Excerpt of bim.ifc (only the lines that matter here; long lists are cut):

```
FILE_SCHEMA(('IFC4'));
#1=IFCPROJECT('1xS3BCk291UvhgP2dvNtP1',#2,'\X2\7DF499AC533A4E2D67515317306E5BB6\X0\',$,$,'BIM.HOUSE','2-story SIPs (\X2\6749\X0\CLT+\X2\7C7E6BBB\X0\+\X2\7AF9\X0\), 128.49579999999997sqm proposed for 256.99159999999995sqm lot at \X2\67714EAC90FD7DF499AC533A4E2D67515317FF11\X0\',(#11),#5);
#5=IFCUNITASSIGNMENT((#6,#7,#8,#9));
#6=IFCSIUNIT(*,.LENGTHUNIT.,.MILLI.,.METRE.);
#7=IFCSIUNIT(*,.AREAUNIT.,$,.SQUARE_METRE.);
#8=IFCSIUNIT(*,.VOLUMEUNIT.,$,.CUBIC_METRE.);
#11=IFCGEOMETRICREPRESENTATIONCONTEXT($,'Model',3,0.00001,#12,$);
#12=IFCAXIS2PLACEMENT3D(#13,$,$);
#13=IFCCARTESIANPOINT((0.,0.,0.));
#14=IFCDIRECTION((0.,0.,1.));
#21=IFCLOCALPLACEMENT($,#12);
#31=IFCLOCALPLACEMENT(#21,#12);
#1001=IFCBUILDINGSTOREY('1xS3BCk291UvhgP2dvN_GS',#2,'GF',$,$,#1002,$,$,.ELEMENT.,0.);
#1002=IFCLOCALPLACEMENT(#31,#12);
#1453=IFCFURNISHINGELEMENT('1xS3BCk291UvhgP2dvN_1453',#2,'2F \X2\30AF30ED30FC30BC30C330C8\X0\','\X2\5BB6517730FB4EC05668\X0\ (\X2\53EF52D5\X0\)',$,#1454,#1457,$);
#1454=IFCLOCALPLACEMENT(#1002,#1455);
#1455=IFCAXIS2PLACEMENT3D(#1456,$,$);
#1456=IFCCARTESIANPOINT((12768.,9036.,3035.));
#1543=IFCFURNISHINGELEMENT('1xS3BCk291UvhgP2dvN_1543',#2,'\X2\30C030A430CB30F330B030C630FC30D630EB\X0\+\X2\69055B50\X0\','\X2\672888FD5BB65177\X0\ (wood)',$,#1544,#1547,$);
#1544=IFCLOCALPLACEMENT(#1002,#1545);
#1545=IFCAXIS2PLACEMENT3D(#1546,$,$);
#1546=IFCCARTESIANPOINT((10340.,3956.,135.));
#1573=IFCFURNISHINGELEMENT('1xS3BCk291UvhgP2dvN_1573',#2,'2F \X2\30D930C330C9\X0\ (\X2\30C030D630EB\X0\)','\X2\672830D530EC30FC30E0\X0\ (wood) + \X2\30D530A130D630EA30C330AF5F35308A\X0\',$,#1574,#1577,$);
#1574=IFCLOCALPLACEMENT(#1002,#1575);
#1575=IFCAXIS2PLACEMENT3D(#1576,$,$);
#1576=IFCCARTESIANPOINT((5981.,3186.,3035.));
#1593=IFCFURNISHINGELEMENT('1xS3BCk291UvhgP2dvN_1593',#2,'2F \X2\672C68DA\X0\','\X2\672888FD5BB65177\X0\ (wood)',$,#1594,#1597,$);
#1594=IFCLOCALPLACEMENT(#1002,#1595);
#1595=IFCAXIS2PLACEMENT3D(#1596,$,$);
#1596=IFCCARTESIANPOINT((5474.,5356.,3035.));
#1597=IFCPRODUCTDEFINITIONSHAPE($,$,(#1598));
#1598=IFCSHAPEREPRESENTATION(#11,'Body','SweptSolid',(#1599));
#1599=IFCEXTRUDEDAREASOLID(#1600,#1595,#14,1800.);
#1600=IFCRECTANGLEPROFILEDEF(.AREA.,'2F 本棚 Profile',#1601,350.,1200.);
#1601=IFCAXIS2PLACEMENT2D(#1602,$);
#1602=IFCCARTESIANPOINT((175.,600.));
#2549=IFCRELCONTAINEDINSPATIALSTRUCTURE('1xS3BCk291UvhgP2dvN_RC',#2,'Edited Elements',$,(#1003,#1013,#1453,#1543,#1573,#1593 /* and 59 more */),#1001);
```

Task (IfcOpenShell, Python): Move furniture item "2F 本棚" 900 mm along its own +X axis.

```python
import ifcopenshell
import ifcopenshell.api.geometry
import ifcopenshell.util.placement

model = ifcopenshell.open("bim.ifc")

item = model.by_id(1593)
matrix = ifcopenshell.util.placement.get_local_placement(item.ObjectPlacement)
matrix[:3, 3] += matrix[:3, 0] * 900.0
ifcopenshell.api.geometry.edit_object_placement(model, product=item, matrix=matrix, is_si=False)

print(ifcopenshell.util.placement.get_local_placement(item.ObjectPlacement).round(3) + 0.0)

model.write("bim-out.ifc")
```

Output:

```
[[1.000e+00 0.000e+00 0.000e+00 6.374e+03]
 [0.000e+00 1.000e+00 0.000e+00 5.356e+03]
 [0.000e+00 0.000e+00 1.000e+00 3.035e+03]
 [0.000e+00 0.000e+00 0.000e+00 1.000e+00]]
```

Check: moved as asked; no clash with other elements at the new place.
